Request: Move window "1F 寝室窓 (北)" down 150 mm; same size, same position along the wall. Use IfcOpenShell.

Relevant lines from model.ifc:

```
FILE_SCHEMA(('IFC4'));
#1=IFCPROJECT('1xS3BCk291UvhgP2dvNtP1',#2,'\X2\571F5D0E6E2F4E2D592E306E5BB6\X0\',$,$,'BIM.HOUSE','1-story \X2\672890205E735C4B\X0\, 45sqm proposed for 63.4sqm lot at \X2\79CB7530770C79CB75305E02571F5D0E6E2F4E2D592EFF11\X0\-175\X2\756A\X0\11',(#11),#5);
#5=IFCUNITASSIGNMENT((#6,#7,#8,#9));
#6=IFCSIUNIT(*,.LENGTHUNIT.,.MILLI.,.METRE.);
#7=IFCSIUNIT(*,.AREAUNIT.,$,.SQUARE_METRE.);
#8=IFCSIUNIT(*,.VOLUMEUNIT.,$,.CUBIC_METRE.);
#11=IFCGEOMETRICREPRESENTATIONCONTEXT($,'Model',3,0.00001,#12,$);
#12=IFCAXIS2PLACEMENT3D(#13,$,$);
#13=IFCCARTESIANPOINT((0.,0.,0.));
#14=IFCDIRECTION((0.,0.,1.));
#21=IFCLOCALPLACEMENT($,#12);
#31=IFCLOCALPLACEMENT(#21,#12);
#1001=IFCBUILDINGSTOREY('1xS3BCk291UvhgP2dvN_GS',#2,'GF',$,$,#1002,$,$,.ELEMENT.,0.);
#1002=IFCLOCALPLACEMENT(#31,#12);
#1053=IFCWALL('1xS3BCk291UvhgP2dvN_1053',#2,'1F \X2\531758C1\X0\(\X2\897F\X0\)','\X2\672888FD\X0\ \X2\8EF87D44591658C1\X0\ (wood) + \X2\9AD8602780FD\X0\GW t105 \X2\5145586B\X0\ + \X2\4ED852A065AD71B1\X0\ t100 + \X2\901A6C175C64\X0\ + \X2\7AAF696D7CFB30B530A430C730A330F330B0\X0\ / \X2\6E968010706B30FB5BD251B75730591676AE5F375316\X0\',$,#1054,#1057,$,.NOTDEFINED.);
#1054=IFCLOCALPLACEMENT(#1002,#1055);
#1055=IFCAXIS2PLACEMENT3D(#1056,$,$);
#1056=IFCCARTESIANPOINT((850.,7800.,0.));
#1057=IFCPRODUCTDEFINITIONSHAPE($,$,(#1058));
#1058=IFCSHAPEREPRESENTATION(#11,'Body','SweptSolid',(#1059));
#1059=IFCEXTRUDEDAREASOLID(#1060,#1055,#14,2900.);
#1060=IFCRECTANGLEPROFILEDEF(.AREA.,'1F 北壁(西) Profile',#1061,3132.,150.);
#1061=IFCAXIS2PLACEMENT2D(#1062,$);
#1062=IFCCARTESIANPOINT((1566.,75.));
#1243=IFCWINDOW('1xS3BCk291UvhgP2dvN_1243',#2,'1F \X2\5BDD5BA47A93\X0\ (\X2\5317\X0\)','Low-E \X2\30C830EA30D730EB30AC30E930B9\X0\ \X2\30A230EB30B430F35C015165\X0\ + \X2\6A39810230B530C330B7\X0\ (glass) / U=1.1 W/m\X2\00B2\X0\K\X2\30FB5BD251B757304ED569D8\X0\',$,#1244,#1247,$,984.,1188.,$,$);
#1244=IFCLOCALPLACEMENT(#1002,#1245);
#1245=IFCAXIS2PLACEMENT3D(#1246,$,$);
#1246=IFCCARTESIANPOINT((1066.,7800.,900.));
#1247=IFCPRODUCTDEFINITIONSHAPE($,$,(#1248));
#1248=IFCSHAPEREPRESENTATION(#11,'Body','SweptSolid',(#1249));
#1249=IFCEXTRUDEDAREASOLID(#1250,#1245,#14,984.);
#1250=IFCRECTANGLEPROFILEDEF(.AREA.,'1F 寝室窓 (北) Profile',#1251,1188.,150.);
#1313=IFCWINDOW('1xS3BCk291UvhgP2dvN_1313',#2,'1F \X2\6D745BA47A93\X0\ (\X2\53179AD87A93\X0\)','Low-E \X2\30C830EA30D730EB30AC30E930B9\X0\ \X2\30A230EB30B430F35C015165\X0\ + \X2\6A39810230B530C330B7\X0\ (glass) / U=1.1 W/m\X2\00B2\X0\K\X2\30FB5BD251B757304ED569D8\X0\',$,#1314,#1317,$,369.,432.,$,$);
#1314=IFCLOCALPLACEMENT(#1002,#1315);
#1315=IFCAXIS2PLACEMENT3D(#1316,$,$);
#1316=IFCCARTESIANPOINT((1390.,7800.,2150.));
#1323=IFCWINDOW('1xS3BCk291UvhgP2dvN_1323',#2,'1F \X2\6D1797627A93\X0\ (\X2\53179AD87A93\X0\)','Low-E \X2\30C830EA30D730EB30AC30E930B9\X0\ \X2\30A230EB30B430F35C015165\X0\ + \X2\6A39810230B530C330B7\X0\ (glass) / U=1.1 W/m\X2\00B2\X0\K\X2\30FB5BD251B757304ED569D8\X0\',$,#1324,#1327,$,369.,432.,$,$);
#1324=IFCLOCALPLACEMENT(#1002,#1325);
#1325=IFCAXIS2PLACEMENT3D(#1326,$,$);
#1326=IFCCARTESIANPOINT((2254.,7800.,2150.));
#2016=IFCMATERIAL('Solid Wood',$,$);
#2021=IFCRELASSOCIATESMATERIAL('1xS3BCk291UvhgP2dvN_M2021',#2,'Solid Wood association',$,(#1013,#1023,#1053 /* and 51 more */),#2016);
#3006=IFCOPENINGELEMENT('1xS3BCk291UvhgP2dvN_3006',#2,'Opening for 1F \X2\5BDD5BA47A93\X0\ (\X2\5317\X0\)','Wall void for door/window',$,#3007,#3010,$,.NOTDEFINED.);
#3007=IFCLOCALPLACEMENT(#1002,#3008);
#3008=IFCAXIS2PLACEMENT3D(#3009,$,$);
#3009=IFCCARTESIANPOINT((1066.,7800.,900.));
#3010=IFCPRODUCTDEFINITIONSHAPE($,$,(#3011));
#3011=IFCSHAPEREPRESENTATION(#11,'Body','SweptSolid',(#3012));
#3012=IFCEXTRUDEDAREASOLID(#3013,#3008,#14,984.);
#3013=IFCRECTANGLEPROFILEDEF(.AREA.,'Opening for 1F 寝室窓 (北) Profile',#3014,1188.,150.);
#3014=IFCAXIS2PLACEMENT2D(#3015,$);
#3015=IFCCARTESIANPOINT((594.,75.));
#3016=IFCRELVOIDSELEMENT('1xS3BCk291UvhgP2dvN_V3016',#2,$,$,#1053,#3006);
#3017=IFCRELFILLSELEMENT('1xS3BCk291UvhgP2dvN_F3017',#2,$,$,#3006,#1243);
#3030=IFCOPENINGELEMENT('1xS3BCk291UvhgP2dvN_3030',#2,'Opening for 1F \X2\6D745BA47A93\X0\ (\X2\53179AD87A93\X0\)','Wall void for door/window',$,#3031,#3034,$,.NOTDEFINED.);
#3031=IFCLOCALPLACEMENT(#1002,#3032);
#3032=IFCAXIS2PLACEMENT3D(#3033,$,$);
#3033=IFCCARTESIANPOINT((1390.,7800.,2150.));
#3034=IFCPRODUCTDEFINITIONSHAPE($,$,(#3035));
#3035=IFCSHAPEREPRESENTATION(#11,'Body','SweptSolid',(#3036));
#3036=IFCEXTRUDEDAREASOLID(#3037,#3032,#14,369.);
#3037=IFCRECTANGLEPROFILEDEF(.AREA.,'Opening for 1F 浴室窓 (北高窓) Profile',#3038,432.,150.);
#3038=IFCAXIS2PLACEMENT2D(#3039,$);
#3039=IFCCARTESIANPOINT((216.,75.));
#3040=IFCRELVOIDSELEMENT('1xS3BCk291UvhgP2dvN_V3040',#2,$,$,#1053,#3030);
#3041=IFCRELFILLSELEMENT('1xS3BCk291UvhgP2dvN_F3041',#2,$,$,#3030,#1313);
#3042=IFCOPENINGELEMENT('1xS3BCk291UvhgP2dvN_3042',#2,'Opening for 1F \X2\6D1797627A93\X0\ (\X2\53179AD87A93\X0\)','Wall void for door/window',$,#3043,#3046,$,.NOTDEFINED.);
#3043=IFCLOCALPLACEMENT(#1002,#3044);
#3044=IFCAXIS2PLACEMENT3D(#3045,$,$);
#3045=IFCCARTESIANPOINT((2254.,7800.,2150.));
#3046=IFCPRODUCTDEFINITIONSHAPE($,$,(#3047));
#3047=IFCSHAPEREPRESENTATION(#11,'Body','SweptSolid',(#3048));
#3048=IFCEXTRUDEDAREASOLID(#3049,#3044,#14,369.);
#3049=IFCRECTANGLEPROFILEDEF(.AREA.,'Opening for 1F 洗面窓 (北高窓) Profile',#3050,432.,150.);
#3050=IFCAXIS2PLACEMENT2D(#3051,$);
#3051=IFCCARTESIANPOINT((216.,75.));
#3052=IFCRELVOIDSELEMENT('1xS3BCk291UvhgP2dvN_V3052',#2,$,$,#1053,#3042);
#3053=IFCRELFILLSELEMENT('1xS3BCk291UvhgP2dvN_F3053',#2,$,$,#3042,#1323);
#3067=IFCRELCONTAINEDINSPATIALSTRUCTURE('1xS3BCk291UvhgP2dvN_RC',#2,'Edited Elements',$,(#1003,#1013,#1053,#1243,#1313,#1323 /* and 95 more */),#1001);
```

```python
import numpy as np
import ifcopenshell
import ifcopenshell.api.geometry
import ifcopenshell.util.placement
import ifcopenshell.util.unit

model = ifcopenshell.open("model.ifc")
unit_scale = ifcopenshell.util.unit.calculate_unit_scale(model)

window = model.by_id(1243)
opening = window.FillsVoids[0].RelatingOpeningElement
dz = -150.0

shift = np.array([0.0, 0.0, dz])
# The window is not placed relative to its opening, so move both.
for product in (opening, window):
    matrix = ifcopenshell.util.placement.get_local_placement(product.ObjectPlacement)
    matrix[:3, 3] += shift
    ifcopenshell.api.geometry.edit_object_placement(model, product=product, matrix=matrix, is_si=False)

print(f"moved by {dz * unit_scale:+.3f} m")

model.write("model_edited.ifc")
```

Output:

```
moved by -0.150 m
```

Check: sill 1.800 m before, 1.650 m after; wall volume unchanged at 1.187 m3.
